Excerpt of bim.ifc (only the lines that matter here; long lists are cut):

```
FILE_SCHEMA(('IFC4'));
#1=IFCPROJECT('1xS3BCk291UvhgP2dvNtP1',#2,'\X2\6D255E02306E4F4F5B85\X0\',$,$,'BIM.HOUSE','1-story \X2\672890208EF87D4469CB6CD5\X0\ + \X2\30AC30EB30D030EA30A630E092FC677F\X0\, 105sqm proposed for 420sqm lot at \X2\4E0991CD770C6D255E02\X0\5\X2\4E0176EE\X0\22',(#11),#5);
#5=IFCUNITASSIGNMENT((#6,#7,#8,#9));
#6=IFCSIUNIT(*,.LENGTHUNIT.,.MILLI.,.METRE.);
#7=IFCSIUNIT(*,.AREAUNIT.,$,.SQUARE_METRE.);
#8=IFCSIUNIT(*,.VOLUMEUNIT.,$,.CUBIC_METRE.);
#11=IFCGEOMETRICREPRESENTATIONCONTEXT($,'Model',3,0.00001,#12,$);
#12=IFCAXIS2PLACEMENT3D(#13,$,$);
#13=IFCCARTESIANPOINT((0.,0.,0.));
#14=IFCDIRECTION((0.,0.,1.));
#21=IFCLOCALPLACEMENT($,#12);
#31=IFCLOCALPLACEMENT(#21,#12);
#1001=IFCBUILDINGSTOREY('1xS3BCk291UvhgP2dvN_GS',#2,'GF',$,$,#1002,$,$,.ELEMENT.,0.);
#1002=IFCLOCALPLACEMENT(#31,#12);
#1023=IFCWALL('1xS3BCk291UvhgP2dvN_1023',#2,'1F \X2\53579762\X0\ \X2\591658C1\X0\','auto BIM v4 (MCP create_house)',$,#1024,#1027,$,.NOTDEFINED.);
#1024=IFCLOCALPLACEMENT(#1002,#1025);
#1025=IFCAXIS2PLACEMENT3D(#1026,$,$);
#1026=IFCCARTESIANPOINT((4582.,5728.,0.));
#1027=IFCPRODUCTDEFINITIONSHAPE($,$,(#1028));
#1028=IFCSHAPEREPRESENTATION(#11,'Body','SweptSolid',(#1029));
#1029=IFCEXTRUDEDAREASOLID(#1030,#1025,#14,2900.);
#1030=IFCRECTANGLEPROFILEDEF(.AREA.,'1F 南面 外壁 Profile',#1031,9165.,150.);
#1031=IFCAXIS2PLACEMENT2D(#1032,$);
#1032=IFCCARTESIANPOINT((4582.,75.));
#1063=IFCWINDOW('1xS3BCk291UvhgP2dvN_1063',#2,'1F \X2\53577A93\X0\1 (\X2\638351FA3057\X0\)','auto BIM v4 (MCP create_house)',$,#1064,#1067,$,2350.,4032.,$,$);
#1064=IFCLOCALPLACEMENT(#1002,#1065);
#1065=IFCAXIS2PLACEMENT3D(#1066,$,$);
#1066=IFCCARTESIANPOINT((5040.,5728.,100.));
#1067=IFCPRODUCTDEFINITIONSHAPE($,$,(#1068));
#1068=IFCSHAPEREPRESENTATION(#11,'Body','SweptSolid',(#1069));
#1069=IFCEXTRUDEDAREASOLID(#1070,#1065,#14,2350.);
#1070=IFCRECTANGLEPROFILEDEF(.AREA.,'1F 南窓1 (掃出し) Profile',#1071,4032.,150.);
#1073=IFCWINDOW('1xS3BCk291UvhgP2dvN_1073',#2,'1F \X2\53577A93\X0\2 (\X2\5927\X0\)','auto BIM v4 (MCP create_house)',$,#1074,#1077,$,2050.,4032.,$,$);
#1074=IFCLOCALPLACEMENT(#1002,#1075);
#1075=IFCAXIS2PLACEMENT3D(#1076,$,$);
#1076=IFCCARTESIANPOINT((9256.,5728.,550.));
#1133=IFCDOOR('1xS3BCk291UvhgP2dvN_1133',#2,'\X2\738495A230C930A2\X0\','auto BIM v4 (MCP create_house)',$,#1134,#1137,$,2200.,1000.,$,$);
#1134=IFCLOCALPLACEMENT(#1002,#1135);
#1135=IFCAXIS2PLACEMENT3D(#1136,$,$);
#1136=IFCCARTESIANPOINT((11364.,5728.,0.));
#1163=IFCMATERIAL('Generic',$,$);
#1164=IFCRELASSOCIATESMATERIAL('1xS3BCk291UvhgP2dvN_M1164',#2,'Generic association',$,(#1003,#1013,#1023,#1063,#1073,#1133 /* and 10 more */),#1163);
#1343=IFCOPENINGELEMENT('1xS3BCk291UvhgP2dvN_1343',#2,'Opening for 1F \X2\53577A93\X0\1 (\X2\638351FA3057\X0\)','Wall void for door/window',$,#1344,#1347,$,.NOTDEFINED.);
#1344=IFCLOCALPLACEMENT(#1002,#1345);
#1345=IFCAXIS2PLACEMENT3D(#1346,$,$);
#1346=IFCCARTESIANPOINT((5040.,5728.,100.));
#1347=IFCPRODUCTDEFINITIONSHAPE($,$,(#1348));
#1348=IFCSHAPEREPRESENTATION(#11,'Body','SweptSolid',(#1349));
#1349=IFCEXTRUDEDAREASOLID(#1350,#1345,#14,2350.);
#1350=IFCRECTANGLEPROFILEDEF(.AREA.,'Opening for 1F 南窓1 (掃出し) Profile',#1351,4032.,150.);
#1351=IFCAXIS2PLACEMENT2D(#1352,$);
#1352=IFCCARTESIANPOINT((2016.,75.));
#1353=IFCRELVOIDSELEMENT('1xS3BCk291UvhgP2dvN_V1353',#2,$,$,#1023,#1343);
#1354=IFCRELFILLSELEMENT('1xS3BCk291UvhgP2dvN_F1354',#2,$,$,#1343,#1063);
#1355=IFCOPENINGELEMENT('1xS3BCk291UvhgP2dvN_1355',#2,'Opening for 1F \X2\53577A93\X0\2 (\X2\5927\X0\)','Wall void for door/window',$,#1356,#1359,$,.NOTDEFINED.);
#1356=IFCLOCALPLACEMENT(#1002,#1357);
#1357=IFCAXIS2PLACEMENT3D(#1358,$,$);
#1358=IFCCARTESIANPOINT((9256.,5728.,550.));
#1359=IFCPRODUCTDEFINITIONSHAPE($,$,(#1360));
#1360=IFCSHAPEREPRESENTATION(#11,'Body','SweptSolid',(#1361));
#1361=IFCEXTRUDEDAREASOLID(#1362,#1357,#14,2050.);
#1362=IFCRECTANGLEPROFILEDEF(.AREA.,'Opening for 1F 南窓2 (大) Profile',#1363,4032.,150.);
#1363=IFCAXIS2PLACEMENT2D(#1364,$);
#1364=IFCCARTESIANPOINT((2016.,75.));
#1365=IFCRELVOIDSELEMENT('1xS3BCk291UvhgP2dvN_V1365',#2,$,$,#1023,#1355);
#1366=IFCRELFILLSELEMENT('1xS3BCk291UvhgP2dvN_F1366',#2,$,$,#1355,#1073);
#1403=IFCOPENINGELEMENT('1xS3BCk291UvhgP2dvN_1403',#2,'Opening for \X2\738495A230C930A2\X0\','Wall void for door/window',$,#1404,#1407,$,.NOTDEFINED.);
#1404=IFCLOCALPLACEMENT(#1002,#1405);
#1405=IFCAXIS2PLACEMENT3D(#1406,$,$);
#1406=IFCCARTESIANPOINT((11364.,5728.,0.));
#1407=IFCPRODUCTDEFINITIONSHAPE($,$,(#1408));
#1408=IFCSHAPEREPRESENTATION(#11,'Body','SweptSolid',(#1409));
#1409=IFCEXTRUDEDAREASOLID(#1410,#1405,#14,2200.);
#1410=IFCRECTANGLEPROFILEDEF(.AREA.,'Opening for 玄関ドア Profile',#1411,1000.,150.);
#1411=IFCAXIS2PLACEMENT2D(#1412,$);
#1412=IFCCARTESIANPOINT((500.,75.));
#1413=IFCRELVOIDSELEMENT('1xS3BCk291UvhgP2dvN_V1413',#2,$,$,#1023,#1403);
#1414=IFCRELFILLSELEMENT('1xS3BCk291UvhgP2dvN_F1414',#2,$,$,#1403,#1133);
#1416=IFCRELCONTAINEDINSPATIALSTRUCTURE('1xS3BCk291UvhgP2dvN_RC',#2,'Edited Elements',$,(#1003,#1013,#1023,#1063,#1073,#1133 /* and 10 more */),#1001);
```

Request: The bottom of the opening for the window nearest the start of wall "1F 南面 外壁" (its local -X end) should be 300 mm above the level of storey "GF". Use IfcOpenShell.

```python
import numpy as np
import ifcopenshell
import ifcopenshell.api.geometry
import ifcopenshell.geom
import ifcopenshell.util.element
import ifcopenshell.util.placement
import ifcopenshell.util.shape
import ifcopenshell.util.unit

model = ifcopenshell.open("bim.ifc")
unit_scale = ifcopenshell.util.unit.calculate_unit_scale(model)

window = model.by_guid("1xS3BCk291UvhgP2dvN_1063")
opening = window.FillsVoids[0].RelatingOpeningElement
storey = ifcopenshell.util.element.get_container(window, ifc_class="IfcBuildingStorey")
level = ifcopenshell.util.placement.get_local_placement(storey.ObjectPlacement)[2, 3]

# The opening's origin need not be at the sill, so measure its lowest point.
shape = ifcopenshell.geom.create_shape(ifcopenshell.geom.settings(), opening)
bottom = ifcopenshell.util.shape.get_shape_bottom_elevation(shape, shape.geometry) / unit_scale
dz = level + 300.0 - bottom

shift = np.array([0.0, 0.0, dz])
# The window is not placed relative to its opening, so move both.
for product in (opening, window):
    matrix = ifcopenshell.util.placement.get_local_placement(product.ObjectPlacement)
    matrix[:3, 3] += shift
    ifcopenshell.api.geometry.edit_object_placement(model, product=product, matrix=matrix, is_si=False)

print(f"moved by {dz * unit_scale:+.3f} m")

model.write("bim_edited.ifc")
```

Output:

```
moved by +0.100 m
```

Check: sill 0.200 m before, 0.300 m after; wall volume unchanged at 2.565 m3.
